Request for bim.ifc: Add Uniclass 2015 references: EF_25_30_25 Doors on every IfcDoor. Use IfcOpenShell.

First a look at what the model holds.

```python
import ifcopenshell

model = ifcopenshell.open("bim.ifc")
print(model.schema)
print("classifications:", [c.Name for c in model.by_type("IfcClassification")])
for ifc_class in ("IfcDoor", "IfcRoof", "IfcStair", "IfcWall", "IfcWindow"):
    print(ifc_class, len(model.by_type(ifc_class)))
```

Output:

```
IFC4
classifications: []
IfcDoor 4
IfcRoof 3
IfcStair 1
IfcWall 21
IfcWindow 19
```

```python
import ifcopenshell
import ifcopenshell.api.classification

model = ifcopenshell.open("bim.ifc")

system = ifcopenshell.api.classification.add_classification(model, classification="Uniclass 2015")

codes = {
    "IfcDoor": ("EF_25_30_25", "Doors"),
}
for ifc_class, (code, name) in codes.items():
    products = model.by_type(ifc_class)
    ifcopenshell.api.classification.add_reference(
        model, products=products, classification=system, identification=code, name=name
    )
    print(code, len(products))

model.write("bim_updated.ifc")
```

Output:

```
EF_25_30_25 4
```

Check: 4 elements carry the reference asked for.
